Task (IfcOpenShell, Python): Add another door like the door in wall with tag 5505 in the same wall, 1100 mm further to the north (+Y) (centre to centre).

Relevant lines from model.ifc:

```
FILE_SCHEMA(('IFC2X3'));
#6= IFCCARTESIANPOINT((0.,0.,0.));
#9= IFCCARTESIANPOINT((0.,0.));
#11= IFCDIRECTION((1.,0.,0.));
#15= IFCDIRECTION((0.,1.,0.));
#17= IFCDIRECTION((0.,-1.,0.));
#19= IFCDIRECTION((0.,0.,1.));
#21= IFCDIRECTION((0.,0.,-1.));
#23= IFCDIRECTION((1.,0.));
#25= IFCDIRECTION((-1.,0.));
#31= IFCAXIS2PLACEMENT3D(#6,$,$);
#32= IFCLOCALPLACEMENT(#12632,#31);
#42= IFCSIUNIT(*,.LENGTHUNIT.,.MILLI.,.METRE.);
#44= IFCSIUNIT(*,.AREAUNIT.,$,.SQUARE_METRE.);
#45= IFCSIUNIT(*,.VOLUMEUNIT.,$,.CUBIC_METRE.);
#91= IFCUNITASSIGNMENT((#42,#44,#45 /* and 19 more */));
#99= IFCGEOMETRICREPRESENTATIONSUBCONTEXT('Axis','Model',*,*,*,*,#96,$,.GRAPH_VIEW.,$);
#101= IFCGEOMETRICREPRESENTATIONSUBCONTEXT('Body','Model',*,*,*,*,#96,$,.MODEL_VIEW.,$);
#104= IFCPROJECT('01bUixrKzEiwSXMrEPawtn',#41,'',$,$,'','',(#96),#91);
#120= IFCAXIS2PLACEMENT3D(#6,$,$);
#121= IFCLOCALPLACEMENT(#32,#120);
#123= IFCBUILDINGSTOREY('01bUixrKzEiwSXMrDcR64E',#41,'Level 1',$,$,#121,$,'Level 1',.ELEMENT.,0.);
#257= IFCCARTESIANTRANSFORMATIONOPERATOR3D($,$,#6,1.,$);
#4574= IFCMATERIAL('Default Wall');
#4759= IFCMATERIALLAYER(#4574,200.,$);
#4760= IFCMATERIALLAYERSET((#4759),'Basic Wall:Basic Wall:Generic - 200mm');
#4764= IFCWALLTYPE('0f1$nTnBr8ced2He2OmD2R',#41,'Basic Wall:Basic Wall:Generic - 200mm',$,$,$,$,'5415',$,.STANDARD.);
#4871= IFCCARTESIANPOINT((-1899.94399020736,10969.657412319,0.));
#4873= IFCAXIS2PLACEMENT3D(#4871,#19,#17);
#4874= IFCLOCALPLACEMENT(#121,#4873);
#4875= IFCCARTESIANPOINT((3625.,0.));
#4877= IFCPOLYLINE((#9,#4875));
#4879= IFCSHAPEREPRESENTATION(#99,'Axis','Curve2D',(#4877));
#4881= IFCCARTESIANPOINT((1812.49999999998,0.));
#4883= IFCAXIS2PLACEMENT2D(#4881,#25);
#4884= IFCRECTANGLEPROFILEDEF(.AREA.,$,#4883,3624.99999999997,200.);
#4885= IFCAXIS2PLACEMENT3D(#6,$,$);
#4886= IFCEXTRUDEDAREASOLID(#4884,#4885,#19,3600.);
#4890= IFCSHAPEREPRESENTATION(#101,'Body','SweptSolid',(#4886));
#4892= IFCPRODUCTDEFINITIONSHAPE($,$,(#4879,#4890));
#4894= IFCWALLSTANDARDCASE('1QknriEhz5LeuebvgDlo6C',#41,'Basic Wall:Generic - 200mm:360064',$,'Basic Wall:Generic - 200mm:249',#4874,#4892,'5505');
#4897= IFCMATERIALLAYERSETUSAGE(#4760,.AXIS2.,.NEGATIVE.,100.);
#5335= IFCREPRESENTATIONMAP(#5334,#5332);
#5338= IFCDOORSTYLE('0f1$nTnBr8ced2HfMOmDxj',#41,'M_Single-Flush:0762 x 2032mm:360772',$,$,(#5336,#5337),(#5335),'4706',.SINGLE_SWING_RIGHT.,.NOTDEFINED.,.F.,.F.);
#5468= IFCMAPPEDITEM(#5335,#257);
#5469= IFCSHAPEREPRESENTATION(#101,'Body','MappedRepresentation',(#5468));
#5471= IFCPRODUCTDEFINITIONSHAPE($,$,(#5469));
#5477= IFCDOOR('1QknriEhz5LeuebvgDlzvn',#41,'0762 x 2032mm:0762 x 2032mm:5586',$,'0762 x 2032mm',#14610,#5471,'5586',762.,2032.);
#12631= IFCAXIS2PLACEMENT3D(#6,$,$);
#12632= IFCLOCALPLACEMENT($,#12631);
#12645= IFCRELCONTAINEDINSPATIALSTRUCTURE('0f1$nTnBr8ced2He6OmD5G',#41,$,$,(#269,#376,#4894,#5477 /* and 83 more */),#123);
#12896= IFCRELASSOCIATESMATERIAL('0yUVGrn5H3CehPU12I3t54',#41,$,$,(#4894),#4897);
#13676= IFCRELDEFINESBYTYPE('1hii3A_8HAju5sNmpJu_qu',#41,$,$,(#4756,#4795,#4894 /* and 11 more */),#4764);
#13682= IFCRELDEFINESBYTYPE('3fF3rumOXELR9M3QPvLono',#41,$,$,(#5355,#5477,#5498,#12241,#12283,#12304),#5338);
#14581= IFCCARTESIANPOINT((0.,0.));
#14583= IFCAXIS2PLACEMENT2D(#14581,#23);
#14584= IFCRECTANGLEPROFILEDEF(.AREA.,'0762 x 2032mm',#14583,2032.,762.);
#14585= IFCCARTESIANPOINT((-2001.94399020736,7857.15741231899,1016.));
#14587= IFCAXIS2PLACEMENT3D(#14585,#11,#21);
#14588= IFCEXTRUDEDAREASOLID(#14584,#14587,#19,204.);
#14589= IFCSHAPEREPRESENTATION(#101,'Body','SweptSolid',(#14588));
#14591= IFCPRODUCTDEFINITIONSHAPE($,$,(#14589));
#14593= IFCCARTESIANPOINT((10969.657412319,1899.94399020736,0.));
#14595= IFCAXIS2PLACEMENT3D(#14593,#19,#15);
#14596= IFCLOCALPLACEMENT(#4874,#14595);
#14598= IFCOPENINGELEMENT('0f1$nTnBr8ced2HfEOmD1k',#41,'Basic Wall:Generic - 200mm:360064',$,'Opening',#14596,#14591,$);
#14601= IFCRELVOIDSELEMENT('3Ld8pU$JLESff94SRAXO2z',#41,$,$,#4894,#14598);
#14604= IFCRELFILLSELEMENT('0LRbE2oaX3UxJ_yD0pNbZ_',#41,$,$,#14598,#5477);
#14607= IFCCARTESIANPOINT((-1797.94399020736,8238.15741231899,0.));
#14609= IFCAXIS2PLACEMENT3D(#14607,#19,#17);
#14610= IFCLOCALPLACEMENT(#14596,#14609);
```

```python
import ifcopenshell
import ifcopenshell.api.feature
import ifcopenshell.api.geometry
import ifcopenshell.api.root
import ifcopenshell.geom
import ifcopenshell.util.element
import ifcopenshell.util.placement
import ifcopenshell.util.shape

model = ifcopenshell.open("model.ifc")
settings = ifcopenshell.geom.settings()


def volume(element):
    """Net volume in cubic metres, openings subtracted."""
    shape = ifcopenshell.geom.create_shape(settings, element)
    return ifcopenshell.util.shape.get_volume(shape.geometry)


def reuse_history(source, copy):
    """copy_class also copies each property set's owner history, people and application; keep the originals."""
    for rel in copy.IsDefinedBy:
        if rel.is_a("IfcRelDefinesByProperties") and (history := rel.RelatingPropertyDefinition.OwnerHistory):
            rel.RelatingPropertyDefinition.OwnerHistory = source.OwnerHistory
            ifcopenshell.util.element.remove_deep2(model, history)


door = model.by_guid("1QknriEhz5LeuebvgDlzvn")
opening = door.FillsVoids[0].RelatingOpeningElement
wall = opening.VoidsElements[0].RelatingBuildingElement
before = volume(wall)
shift = ifcopenshell.util.placement.get_local_placement(wall.ObjectPlacement)[:3, 0] * -1100.0

# copy_class copies the void relationship, type, container and properties, but no geometry.
new_opening = ifcopenshell.api.root.copy_class(model, product=opening)
new_opening.Representation = ifcopenshell.util.element.copy_deep(
    model, opening.Representation, exclude=["IfcGeometricRepresentationContext", "IfcRepresentationMap"]
)
new_opening.Name = "Basic Wall:Generic - 200mm"
new_door = ifcopenshell.api.root.copy_class(model, product=door)
new_door.Representation = ifcopenshell.util.element.copy_deep(
    model, door.Representation, exclude=["IfcGeometricRepresentationContext", "IfcRepresentationMap"]
)
new_door.Name = "0762 x 2032mm:0762 x 2032mm"
new_door.Tag = None
reuse_history(door, new_door)
fills = ifcopenshell.api.feature.add_filling(model, opening=new_opening, element=new_door)
fills.OwnerHistory = new_door.OwnerHistory  # required in IFC2X3

for old, new in ((opening, new_opening), (door, new_door)):
    matrix = ifcopenshell.util.placement.get_local_placement(old.ObjectPlacement)
    matrix[:3, 3] += shift
    ifcopenshell.api.geometry.edit_object_placement(model, product=new, matrix=matrix, is_si=False)

after = volume(wall)

print(f"wall volume {before:.3f} -> {after:.3f} m3")

model.write("model_v2.ifc")
```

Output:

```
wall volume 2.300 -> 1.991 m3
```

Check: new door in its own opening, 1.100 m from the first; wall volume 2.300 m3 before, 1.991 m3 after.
